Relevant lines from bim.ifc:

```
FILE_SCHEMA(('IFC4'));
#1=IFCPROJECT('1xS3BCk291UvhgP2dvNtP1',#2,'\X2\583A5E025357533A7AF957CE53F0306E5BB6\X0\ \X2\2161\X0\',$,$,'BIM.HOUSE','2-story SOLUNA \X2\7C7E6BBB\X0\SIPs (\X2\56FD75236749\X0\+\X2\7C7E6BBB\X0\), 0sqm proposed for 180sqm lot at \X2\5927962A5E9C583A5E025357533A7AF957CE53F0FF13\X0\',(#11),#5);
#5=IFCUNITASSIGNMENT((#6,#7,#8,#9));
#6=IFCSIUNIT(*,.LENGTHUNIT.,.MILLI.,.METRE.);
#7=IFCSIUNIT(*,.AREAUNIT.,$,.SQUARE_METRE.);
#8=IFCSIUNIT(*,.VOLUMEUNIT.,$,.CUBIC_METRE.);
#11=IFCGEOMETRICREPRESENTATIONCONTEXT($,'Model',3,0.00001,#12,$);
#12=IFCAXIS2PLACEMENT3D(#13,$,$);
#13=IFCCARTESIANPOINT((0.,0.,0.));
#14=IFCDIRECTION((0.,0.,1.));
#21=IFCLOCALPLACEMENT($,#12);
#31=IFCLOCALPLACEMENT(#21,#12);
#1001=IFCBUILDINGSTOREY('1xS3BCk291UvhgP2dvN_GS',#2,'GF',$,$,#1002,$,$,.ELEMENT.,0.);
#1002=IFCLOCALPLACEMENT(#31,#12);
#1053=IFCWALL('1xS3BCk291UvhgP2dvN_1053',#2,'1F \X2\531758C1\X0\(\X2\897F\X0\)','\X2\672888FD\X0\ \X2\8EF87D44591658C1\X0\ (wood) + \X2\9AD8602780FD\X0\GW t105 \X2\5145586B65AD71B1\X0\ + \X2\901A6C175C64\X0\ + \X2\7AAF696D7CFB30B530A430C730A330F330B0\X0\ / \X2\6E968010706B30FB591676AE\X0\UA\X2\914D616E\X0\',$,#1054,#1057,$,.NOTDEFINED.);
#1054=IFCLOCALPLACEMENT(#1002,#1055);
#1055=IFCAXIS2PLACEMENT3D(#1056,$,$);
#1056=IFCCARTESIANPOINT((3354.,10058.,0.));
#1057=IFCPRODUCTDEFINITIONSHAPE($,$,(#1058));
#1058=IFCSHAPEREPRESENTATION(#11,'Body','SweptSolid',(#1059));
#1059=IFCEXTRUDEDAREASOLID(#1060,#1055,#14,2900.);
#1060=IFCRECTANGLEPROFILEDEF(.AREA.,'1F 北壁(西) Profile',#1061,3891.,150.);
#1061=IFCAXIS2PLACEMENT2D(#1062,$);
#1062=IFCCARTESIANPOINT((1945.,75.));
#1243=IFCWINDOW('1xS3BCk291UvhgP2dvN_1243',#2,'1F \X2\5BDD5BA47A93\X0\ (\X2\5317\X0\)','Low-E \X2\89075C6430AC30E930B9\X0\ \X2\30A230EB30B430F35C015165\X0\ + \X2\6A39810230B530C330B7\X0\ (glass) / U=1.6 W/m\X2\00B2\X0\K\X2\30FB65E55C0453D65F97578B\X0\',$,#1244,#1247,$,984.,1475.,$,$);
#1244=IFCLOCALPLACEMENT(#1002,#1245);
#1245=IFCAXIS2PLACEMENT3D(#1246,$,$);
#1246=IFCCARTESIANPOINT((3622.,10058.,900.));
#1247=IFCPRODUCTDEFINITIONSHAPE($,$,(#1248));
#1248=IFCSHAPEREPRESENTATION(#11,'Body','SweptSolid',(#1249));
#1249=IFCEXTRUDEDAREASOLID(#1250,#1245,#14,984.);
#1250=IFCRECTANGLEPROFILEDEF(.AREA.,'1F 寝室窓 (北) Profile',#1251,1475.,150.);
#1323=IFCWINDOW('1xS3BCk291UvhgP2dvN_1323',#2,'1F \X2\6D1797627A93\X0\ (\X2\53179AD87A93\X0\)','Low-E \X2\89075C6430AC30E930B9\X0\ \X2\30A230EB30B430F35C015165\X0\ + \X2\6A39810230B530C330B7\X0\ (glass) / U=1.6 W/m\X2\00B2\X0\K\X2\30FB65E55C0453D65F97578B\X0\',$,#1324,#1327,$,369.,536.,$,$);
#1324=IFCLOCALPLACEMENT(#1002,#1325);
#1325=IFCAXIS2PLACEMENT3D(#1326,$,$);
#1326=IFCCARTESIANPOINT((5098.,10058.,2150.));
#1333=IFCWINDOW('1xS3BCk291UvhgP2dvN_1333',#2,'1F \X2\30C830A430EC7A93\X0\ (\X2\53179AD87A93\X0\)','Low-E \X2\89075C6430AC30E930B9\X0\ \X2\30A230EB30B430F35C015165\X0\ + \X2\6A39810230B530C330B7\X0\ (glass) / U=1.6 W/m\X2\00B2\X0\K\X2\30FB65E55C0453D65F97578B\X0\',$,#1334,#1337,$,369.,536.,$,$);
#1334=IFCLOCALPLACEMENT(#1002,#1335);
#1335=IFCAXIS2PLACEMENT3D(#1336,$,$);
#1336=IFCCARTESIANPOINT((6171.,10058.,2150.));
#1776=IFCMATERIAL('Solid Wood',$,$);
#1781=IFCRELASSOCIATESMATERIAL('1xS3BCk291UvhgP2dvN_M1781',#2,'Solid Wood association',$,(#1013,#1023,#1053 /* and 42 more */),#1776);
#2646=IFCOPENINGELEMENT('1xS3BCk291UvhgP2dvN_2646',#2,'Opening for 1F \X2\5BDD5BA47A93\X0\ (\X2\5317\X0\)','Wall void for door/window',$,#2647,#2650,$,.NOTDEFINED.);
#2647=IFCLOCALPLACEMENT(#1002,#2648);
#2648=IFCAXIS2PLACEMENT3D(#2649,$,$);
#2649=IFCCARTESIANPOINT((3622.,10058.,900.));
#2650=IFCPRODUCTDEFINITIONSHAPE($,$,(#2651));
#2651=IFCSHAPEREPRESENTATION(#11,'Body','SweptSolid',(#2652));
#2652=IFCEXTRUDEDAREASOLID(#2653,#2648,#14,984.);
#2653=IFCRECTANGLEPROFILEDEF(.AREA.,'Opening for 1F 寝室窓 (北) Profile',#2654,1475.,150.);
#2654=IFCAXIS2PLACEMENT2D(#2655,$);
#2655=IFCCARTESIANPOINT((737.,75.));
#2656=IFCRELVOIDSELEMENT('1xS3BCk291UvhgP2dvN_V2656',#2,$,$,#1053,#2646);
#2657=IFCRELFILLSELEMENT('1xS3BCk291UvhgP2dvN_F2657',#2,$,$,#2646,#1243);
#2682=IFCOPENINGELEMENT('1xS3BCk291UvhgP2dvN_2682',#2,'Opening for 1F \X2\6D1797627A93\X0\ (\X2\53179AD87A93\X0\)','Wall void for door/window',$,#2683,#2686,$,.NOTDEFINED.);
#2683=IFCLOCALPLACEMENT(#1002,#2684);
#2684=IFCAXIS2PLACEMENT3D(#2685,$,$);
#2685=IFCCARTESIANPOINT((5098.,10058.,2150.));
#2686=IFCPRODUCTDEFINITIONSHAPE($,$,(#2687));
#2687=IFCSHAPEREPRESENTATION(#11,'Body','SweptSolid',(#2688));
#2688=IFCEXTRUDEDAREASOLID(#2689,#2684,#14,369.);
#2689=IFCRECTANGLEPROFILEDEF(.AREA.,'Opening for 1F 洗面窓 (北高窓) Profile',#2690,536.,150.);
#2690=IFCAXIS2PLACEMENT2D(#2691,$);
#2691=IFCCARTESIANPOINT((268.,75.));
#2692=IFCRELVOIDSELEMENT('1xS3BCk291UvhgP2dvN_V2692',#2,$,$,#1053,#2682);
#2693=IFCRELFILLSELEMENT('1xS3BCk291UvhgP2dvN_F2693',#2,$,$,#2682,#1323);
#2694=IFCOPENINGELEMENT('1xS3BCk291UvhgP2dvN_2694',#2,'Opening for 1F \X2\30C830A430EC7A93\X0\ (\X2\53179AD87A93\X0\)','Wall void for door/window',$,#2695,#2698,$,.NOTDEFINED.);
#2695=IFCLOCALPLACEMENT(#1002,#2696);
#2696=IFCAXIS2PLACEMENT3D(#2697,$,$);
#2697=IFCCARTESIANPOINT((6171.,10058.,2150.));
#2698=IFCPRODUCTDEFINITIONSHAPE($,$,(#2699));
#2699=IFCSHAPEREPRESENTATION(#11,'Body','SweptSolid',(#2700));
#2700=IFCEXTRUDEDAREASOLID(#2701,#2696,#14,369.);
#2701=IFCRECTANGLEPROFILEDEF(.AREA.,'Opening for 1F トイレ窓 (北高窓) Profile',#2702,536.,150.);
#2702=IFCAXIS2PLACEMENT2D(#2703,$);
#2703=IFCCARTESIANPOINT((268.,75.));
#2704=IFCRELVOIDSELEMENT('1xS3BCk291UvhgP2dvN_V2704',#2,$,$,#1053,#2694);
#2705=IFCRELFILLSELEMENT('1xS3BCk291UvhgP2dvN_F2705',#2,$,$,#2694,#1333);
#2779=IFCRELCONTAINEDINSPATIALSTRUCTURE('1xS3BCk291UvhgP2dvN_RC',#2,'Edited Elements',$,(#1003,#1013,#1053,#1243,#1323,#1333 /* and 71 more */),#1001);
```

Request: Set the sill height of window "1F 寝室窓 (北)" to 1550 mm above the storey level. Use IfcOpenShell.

```python
import numpy as np
import ifcopenshell
import ifcopenshell.api.geometry
import ifcopenshell.geom
import ifcopenshell.util.element
import ifcopenshell.util.placement
import ifcopenshell.util.shape
import ifcopenshell.util.unit

model = ifcopenshell.open("bim.ifc")
unit_scale = ifcopenshell.util.unit.calculate_unit_scale(model)

window = model.by_guid("1xS3BCk291UvhgP2dvN_1243")
opening = window.FillsVoids[0].RelatingOpeningElement
storey = ifcopenshell.util.element.get_container(window, ifc_class="IfcBuildingStorey")
level = ifcopenshell.util.placement.get_local_placement(storey.ObjectPlacement)[2, 3]

# The opening's origin need not be at the sill, so measure its lowest point.
shape = ifcopenshell.geom.create_shape(ifcopenshell.geom.settings(), opening)
bottom = ifcopenshell.util.shape.get_shape_bottom_elevation(shape, shape.geometry) / unit_scale
dz = level + 1.55 / unit_scale - bottom

shift = np.array([0.0, 0.0, dz])
# The window is not placed relative to its opening, so move both.
for product in (opening, window):
    matrix = ifcopenshell.util.placement.get_local_placement(product.ObjectPlacement)
    matrix[:3, 3] += shift
    ifcopenshell.api.geometry.edit_object_placement(model, product=product, matrix=matrix, is_si=False)

print(f"moved by {dz * unit_scale:+.3f} m")

model.write("bim_updated.ifc")
```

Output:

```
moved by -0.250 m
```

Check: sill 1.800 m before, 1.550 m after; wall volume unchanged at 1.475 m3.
